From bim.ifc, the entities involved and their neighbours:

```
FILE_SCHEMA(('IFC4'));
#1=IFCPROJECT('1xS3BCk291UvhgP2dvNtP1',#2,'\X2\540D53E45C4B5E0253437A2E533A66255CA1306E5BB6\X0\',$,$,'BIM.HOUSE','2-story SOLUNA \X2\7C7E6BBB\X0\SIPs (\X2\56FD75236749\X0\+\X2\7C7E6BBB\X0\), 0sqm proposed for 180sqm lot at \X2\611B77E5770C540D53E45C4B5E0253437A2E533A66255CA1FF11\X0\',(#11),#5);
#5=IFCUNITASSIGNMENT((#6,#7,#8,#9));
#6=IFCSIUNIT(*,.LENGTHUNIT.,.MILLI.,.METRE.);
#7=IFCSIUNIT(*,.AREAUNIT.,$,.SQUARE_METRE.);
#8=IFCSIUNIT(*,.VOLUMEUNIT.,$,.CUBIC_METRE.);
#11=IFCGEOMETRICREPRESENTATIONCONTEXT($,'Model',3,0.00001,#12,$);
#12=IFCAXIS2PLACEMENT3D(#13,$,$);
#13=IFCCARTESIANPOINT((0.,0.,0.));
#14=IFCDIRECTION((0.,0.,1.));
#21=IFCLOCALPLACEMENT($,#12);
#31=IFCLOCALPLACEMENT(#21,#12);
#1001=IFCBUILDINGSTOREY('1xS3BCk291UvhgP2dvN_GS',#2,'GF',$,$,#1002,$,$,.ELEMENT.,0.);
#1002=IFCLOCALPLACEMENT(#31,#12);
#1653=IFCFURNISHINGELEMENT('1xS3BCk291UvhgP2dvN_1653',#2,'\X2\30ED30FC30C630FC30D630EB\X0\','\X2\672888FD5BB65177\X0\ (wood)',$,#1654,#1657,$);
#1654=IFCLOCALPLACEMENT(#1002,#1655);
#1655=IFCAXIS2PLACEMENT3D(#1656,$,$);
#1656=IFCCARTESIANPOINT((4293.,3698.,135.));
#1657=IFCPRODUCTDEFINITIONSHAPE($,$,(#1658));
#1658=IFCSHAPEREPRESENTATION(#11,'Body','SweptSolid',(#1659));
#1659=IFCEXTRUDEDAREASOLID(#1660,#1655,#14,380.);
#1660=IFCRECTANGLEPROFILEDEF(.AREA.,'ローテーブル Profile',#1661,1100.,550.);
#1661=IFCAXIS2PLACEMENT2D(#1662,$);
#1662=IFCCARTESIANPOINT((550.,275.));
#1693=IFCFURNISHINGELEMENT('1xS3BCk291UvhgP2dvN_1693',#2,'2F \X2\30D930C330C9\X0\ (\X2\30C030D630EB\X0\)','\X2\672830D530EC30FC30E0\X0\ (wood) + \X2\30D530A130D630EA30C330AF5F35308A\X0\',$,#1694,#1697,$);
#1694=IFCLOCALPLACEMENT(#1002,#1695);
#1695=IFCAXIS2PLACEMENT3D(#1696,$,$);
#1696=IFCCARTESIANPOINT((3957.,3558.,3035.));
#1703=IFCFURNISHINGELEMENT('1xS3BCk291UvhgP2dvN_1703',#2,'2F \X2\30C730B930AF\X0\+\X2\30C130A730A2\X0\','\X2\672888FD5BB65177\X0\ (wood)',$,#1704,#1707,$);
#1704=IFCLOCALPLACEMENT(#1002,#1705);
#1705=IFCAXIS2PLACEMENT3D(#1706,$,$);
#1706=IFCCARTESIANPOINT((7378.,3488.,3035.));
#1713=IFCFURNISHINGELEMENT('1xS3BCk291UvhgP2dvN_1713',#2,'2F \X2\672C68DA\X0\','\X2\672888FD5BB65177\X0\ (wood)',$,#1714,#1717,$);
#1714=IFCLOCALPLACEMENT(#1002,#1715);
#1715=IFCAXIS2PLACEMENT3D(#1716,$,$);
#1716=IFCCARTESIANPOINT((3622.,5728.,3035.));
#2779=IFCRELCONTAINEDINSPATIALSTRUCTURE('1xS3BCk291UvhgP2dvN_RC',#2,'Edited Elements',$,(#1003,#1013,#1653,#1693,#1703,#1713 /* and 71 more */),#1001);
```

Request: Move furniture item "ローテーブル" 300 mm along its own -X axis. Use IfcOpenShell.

```python
import ifcopenshell
import ifcopenshell.api.geometry
import ifcopenshell.util.placement

model = ifcopenshell.open("bim.ifc")

item = model.by_id(1653)
matrix = ifcopenshell.util.placement.get_local_placement(item.ObjectPlacement)
matrix[:3, 3] -= matrix[:3, 0] * 300.0
ifcopenshell.api.geometry.edit_object_placement(model, product=item, matrix=matrix, is_si=False)

print(ifcopenshell.util.placement.get_local_placement(item.ObjectPlacement).round(3) + 0.0)

model.write("bim_rev.ifc")
```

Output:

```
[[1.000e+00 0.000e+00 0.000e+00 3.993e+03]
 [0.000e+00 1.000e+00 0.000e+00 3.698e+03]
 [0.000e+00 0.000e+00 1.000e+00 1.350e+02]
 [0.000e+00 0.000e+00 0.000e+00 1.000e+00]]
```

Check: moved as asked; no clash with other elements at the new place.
